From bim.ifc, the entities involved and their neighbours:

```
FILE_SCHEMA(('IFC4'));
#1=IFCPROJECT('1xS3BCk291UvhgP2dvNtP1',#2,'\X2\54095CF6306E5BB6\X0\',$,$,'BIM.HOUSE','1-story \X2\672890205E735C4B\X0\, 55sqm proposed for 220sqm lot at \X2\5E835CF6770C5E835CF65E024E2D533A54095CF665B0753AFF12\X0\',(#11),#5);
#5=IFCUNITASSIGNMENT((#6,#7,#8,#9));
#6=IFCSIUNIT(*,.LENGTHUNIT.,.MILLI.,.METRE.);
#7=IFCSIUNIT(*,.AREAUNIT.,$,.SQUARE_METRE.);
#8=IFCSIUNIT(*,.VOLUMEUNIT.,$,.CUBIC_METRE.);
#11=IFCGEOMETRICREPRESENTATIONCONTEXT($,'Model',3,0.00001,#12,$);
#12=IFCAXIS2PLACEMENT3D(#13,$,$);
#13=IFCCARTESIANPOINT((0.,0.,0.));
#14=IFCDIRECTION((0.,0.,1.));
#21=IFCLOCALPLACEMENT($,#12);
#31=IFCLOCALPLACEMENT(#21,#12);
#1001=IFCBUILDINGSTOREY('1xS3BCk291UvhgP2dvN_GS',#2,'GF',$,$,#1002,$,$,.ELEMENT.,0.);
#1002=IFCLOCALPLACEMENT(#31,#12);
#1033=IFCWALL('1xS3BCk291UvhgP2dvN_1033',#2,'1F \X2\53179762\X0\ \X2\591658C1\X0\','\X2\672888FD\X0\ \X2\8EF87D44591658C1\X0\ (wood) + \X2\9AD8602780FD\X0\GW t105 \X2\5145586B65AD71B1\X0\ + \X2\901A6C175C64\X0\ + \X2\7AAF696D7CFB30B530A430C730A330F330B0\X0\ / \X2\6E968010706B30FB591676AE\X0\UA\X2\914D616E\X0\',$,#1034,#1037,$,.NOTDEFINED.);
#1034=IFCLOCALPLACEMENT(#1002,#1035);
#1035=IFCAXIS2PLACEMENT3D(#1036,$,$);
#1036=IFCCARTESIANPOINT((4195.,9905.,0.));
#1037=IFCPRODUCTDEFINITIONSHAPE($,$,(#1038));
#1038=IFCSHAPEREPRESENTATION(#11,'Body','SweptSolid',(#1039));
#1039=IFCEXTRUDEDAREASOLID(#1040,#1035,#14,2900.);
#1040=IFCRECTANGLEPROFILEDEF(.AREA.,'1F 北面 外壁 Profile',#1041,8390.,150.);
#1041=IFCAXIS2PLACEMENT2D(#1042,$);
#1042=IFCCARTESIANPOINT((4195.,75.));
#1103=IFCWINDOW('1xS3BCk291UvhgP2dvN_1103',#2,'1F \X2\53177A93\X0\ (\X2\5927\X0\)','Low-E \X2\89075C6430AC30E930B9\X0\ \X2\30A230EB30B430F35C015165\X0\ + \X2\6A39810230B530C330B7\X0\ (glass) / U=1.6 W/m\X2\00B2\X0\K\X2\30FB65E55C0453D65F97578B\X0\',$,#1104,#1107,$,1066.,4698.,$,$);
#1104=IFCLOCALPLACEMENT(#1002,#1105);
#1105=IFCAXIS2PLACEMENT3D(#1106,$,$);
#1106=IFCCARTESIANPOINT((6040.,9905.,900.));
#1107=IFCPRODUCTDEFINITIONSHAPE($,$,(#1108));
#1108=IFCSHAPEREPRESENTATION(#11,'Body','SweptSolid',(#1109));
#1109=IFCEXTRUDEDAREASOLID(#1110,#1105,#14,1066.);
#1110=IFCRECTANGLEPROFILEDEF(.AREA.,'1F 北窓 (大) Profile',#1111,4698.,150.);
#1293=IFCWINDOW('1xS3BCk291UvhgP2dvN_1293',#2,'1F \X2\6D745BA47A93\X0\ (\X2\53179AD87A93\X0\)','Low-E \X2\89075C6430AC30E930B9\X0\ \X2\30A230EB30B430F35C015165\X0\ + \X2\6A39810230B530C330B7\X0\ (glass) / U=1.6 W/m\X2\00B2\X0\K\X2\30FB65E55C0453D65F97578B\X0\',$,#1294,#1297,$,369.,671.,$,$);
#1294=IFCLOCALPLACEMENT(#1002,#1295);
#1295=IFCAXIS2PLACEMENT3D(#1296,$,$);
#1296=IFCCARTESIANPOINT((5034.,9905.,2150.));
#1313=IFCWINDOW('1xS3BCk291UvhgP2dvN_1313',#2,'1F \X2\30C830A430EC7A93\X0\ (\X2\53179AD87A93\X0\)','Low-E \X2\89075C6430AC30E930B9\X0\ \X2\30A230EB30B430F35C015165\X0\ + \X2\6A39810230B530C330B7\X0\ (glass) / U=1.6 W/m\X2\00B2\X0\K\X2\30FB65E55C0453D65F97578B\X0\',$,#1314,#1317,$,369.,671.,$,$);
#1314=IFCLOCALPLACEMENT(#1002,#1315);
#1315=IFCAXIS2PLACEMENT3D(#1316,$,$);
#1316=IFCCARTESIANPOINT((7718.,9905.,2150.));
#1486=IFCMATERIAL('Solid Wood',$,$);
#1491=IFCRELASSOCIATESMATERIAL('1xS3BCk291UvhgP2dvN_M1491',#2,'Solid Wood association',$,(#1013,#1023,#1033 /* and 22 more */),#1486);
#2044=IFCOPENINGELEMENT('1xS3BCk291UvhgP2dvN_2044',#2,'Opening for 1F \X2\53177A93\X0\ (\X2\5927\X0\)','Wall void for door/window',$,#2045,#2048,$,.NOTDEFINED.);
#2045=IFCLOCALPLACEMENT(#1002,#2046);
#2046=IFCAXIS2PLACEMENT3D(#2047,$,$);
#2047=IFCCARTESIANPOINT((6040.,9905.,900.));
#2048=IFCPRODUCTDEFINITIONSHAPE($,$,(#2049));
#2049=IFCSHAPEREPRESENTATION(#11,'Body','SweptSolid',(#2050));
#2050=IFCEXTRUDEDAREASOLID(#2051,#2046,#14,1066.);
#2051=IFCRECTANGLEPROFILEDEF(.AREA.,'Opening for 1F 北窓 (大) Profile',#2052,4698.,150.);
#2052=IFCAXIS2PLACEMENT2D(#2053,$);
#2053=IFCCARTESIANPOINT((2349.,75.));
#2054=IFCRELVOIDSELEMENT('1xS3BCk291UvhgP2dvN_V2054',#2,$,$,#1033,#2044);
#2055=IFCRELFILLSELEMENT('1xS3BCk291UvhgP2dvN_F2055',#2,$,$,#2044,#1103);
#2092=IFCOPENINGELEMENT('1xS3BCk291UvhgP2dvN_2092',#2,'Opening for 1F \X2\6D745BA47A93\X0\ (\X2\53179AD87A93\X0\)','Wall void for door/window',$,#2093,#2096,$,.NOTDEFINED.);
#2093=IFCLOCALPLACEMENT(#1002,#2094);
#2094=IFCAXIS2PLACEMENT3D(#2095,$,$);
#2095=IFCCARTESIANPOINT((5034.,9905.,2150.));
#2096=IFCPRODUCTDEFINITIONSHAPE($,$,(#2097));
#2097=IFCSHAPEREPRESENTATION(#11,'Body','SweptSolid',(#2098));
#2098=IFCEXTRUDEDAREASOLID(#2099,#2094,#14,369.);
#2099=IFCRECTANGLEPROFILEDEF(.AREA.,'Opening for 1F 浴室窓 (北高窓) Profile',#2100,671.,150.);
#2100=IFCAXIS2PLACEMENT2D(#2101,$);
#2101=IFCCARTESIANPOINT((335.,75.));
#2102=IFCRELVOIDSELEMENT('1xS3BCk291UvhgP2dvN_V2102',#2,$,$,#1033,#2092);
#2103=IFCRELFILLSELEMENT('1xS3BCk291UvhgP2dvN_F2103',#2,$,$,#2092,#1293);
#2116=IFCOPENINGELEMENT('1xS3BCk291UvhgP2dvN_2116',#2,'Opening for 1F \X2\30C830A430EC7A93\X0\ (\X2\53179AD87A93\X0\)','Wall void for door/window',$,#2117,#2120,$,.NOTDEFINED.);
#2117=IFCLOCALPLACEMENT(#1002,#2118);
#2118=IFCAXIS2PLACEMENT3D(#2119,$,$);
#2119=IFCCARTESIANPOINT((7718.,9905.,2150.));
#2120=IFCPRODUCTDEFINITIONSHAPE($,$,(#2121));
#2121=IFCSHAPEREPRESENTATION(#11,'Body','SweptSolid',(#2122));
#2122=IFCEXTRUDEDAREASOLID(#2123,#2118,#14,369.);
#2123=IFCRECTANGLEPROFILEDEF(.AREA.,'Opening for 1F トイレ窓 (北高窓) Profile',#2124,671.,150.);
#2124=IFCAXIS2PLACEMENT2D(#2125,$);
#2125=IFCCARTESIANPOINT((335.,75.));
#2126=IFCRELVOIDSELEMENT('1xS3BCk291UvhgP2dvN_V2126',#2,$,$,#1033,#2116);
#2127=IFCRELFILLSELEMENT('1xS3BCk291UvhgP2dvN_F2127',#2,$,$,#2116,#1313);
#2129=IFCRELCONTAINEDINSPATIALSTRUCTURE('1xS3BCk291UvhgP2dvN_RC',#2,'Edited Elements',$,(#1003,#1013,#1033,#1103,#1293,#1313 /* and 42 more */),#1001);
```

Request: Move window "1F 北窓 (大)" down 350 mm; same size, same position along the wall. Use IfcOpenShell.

```python
import numpy as np
import ifcopenshell
import ifcopenshell.api.geometry
import ifcopenshell.util.placement
import ifcopenshell.util.unit

model = ifcopenshell.open("bim.ifc")
unit_scale = ifcopenshell.util.unit.calculate_unit_scale(model)

window = model.by_guid("1xS3BCk291UvhgP2dvN_1103")
opening = window.FillsVoids[0].RelatingOpeningElement
dz = -350.0

shift = np.array([0.0, 0.0, dz])
# The window is not placed relative to its opening, so move both.
for product in (opening, window):
    matrix = ifcopenshell.util.placement.get_local_placement(product.ObjectPlacement)
    matrix[:3, 3] += shift
    ifcopenshell.api.geometry.edit_object_placement(model, product=product, matrix=matrix, is_si=False)

print(f"moved by {dz * unit_scale:+.3f} m")

model.write("bim_updated.ifc")
```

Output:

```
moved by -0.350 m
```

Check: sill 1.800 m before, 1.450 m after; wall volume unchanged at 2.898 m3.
